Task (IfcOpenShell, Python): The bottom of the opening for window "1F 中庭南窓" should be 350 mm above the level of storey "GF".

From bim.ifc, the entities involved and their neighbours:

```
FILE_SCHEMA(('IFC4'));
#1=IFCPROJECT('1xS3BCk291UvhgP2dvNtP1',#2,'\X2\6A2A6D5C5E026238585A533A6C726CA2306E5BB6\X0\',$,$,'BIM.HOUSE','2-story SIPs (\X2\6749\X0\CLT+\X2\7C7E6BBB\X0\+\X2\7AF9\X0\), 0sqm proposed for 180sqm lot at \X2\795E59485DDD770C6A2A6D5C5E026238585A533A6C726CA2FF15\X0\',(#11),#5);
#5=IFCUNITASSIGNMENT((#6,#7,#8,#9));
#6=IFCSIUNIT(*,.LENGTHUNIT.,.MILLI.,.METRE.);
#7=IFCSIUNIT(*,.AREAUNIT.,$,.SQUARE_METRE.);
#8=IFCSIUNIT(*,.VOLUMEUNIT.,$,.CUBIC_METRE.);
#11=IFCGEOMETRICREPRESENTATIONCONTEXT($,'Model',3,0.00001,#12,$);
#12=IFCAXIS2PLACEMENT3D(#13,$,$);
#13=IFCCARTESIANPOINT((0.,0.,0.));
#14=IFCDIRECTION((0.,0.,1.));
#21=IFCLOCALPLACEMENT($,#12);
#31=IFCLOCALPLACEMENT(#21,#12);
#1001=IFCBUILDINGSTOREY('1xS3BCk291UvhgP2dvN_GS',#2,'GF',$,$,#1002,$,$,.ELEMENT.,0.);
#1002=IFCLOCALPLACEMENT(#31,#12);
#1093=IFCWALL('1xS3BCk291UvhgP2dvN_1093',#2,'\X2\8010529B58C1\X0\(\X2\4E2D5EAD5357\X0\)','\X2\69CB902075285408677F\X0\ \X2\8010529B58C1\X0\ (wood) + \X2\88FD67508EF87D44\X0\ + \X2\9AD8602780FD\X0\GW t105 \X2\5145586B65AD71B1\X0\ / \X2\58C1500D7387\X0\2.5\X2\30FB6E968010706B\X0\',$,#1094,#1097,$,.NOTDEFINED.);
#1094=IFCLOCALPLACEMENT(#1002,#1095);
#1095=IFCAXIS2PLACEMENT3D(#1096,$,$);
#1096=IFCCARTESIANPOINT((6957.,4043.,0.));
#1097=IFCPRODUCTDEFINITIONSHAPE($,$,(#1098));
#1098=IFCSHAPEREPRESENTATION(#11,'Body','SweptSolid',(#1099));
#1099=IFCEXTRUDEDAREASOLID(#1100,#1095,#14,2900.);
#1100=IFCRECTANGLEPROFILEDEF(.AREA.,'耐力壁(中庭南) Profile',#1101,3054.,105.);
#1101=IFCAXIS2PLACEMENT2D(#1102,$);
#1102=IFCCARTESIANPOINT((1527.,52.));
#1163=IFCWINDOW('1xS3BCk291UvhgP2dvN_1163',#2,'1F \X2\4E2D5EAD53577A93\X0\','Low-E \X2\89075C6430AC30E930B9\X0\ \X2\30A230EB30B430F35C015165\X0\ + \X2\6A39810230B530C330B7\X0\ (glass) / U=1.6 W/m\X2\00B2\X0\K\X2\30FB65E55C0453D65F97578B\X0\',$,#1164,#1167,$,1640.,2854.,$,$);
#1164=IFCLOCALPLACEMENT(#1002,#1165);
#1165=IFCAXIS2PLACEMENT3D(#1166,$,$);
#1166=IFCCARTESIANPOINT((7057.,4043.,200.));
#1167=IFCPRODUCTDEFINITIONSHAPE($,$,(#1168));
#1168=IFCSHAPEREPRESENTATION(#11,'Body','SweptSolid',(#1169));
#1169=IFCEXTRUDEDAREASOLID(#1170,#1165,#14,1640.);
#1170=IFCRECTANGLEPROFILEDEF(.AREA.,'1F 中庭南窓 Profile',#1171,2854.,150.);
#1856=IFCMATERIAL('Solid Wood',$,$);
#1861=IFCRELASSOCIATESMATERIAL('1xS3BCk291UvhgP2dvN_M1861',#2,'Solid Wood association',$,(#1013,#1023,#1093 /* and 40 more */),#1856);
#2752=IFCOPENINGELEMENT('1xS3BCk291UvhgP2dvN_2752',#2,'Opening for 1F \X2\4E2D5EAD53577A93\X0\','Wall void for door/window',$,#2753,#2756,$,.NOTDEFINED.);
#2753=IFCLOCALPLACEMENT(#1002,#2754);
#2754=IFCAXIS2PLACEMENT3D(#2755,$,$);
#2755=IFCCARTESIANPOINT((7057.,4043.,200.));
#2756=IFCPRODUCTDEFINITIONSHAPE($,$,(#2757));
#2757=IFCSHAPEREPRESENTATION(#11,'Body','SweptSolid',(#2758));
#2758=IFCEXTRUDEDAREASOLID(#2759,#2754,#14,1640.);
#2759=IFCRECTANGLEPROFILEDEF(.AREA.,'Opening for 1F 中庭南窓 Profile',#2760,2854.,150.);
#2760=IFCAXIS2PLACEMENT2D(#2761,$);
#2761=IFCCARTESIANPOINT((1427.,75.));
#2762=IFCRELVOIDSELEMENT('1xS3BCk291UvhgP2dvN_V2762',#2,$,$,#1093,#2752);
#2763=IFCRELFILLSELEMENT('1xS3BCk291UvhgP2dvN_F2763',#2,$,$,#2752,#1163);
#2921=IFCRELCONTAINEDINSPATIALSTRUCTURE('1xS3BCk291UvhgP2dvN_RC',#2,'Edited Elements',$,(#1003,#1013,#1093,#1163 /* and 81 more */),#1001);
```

```python
import numpy as np
import ifcopenshell
import ifcopenshell.api.geometry
import ifcopenshell.geom
import ifcopenshell.util.element
import ifcopenshell.util.placement
import ifcopenshell.util.shape
import ifcopenshell.util.unit

model = ifcopenshell.open("bim.ifc")
unit_scale = ifcopenshell.util.unit.calculate_unit_scale(model)

window = model.by_guid("1xS3BCk291UvhgP2dvN_1163")
opening = window.FillsVoids[0].RelatingOpeningElement
storey = ifcopenshell.util.element.get_container(window, ifc_class="IfcBuildingStorey")
level = ifcopenshell.util.placement.get_local_placement(storey.ObjectPlacement)[2, 3]

# The opening's origin need not be at the sill, so measure its lowest point.
shape = ifcopenshell.geom.create_shape(ifcopenshell.geom.settings(), opening)
bottom = ifcopenshell.util.shape.get_shape_bottom_elevation(shape, shape.geometry) / unit_scale
dz = level + 0.35 / unit_scale - bottom

shift = np.array([0.0, 0.0, dz])
# The window is not placed relative to its opening, so move both.
for product in (opening, window):
    matrix = ifcopenshell.util.placement.get_local_placement(product.ObjectPlacement)
    matrix[:3, 3] += shift
    ifcopenshell.api.geometry.edit_object_placement(model, product=product, matrix=matrix, is_si=False)

print(f"moved by {dz * unit_scale:+.3f} m")

model.write("bim_updated.ifc")
```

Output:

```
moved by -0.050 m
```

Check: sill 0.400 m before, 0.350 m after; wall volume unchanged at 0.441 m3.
